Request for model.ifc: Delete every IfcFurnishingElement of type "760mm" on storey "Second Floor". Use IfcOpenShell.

First a look at what the model holds.

```python
import ifcopenshell
import ifcopenshell.util.element

model = ifcopenshell.open("model.ifc")
print(model.schema)
storey = next(s for s in model.by_type("IfcBuildingStorey") if s.Name == "Second Floor")
furniture = [e for e in ifcopenshell.util.element.get_decomposition(storey) if e.is_a("IfcFurnishingElement")]
seen = {}
for e in furniture:
    element_type = ifcopenshell.util.element.get_type(e)
    name = element_type.Name if element_type not in (None, e) else None
    seen[name] = seen.get(name, 0) + 1
for name, count in sorted(seen.items(), key=str):
    print(count, "x", name)
```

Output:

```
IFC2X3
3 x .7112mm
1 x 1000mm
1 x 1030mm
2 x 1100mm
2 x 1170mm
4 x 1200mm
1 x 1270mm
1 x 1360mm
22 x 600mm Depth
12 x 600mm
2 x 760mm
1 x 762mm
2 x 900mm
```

```python
import ifcopenshell
import ifcopenshell.api.root
import ifcopenshell.util.element

model = ifcopenshell.open("model.ifc")

storey = next(s for s in model.by_type("IfcBuildingStorey") if s.Name == "Second Floor")
furniture = [e for e in ifcopenshell.util.element.get_decomposition(storey) if e.is_a("IfcFurnishingElement")]
targets = [e for e in furniture if (t := ifcopenshell.util.element.get_type(e)) not in (None, e) and t.Name == "760mm"]

for e in targets:
    ifcopenshell.api.root.remove_product(model, product=e)
print(len(targets), "removed")

model.write("model_edited.ifc")
```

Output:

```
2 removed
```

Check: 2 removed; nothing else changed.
